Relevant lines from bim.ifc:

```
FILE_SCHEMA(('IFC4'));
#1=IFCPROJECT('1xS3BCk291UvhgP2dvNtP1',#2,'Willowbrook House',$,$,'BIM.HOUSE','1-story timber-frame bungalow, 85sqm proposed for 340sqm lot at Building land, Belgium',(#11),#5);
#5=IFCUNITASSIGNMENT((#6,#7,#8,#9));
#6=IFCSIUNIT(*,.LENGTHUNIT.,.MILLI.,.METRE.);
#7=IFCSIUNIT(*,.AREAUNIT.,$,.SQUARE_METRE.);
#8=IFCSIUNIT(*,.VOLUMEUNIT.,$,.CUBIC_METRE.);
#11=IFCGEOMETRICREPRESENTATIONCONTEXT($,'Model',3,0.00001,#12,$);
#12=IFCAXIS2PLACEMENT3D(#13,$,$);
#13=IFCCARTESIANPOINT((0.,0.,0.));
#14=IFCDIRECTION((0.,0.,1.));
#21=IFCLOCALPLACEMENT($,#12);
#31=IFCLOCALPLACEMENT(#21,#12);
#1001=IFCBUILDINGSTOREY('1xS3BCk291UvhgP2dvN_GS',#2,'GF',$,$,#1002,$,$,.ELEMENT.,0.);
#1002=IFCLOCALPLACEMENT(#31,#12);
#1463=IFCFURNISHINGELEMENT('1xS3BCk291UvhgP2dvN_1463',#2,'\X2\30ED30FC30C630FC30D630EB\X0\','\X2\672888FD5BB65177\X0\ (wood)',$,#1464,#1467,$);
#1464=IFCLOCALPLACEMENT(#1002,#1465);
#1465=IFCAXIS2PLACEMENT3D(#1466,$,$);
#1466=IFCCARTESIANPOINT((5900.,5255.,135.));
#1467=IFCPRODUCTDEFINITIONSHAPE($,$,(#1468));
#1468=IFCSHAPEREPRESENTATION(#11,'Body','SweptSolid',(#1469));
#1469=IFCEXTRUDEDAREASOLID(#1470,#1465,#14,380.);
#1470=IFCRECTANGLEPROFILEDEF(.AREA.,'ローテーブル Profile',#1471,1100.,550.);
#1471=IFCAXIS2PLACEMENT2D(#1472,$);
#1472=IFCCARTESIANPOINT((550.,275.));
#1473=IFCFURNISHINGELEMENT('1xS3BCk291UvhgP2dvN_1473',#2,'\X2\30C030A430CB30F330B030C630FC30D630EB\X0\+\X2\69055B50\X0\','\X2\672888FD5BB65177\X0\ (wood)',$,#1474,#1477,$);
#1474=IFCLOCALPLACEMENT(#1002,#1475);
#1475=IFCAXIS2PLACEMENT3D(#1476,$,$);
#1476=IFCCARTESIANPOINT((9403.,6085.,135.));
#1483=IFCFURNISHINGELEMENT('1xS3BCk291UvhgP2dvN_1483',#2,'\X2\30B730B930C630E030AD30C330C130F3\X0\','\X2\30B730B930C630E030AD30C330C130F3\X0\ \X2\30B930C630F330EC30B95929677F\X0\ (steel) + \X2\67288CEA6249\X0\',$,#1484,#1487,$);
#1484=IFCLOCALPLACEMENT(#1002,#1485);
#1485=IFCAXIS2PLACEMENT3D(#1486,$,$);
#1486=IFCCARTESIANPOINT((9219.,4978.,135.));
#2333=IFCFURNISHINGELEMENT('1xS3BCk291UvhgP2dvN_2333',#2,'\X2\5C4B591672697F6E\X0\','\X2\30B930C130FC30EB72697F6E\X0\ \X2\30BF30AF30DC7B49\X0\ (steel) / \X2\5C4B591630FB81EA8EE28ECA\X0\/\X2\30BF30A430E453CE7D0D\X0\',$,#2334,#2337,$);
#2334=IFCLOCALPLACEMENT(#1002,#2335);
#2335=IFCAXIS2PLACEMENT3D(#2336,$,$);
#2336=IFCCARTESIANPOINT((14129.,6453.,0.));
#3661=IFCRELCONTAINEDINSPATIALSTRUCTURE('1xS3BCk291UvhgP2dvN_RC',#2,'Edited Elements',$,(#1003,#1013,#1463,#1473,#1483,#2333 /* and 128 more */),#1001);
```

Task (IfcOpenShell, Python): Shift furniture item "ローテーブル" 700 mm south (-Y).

```python
import ifcopenshell
import ifcopenshell.api.geometry
import ifcopenshell.util.placement
import ifcopenshell.util.unit

model = ifcopenshell.open("bim.ifc")
unit_scale = ifcopenshell.util.unit.calculate_unit_scale(model)

item = model.by_guid("1xS3BCk291UvhgP2dvN_1463")
matrix = ifcopenshell.util.placement.get_local_placement(item.ObjectPlacement)
matrix[1, 3] -= 0.7 / unit_scale
ifcopenshell.api.geometry.edit_object_placement(model, product=item, matrix=matrix, is_si=False)

print(ifcopenshell.util.placement.get_local_placement(item.ObjectPlacement).round(3) + 0.0)

model.write("bim_edited.ifc")
```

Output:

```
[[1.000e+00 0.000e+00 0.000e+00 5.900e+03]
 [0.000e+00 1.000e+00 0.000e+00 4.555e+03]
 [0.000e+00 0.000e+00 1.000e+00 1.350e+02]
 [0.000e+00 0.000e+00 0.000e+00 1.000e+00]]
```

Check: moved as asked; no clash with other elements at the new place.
